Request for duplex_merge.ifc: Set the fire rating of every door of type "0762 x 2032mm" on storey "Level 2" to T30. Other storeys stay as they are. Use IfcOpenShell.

First a look at what the model holds.

```python
import ifcopenshell
import ifcopenshell.util.element

model = ifcopenshell.open("duplex_merge.ifc")
print(model.schema)
storey = next(s for s in model.by_type("IfcBuildingStorey") if s.Name == "Level 2")
doors = [e for e in ifcopenshell.util.element.get_decomposition(storey) if e.is_a("IfcDoor")]
seen = {}
for e in doors:
    element_type = ifcopenshell.util.element.get_type(e)
    key = (element_type.Name if element_type != e and element_type else None, ifcopenshell.util.element.get_pset(e, "Pset_DoorCommon", "FireRating"))
    seen[key] = seen.get(key, 0) + 1
for (name, value), count in sorted(seen.items(), key=str):
    print(count, "x", name, "|", value)
```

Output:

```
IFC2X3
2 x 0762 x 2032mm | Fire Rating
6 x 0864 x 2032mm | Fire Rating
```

```python
import ifcopenshell
import ifcopenshell.api.pset
import ifcopenshell.util.element

model = ifcopenshell.open("duplex_merge.ifc")

storey = next(s for s in model.by_type("IfcBuildingStorey") if s.Name == "Level 2")
doors = [e for e in ifcopenshell.util.element.get_decomposition(storey) if e.is_a("IfcDoor")]

count = 0
for e in doors:
    element_type = ifcopenshell.util.element.get_type(e)
    if element_type in (None, e) or element_type.Name != "0762 x 2032mm":
        continue
    # add_pset returns the element's existing set when there is one.
    pset = ifcopenshell.api.pset.add_pset(model, product=e, name="Pset_DoorCommon")
    ifcopenshell.api.pset.edit_pset(model, pset=pset, properties={"FireRating": "T30"})
    count += 1

print(count, "doors updated")

model.write("duplex_merge-out.ifc")
```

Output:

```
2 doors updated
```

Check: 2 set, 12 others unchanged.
